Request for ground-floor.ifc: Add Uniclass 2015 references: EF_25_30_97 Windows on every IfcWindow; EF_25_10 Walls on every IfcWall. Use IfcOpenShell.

First a look at what the model holds.

```python
import ifcopenshell

model = ifcopenshell.open("ground-floor.ifc")
print(model.schema)
print("classifications:", [c.Name for c in model.by_type("IfcClassification")])
for ifc_class in ("IfcDoor", "IfcRoof", "IfcStair", "IfcWall", "IfcWindow"):
    print(ifc_class, len(model.by_type(ifc_class)))
```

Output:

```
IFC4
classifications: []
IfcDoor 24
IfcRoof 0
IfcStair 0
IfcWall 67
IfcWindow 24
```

```python
import ifcopenshell
import ifcopenshell.api.classification

model = ifcopenshell.open("ground-floor.ifc")

system = ifcopenshell.api.classification.add_classification(model, classification="Uniclass 2015")

codes = {
    "IfcWindow": ("EF_25_30_97", "Windows"),
    "IfcWall": ("EF_25_10", "Walls"),
}
for ifc_class, (code, name) in codes.items():
    products = model.by_type(ifc_class)
    ifcopenshell.api.classification.add_reference(
        model, products=products, classification=system, identification=code, name=name
    )
    print(code, len(products))

model.write("ground-floor_edited.ifc")
```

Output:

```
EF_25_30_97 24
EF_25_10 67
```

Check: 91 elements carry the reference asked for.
